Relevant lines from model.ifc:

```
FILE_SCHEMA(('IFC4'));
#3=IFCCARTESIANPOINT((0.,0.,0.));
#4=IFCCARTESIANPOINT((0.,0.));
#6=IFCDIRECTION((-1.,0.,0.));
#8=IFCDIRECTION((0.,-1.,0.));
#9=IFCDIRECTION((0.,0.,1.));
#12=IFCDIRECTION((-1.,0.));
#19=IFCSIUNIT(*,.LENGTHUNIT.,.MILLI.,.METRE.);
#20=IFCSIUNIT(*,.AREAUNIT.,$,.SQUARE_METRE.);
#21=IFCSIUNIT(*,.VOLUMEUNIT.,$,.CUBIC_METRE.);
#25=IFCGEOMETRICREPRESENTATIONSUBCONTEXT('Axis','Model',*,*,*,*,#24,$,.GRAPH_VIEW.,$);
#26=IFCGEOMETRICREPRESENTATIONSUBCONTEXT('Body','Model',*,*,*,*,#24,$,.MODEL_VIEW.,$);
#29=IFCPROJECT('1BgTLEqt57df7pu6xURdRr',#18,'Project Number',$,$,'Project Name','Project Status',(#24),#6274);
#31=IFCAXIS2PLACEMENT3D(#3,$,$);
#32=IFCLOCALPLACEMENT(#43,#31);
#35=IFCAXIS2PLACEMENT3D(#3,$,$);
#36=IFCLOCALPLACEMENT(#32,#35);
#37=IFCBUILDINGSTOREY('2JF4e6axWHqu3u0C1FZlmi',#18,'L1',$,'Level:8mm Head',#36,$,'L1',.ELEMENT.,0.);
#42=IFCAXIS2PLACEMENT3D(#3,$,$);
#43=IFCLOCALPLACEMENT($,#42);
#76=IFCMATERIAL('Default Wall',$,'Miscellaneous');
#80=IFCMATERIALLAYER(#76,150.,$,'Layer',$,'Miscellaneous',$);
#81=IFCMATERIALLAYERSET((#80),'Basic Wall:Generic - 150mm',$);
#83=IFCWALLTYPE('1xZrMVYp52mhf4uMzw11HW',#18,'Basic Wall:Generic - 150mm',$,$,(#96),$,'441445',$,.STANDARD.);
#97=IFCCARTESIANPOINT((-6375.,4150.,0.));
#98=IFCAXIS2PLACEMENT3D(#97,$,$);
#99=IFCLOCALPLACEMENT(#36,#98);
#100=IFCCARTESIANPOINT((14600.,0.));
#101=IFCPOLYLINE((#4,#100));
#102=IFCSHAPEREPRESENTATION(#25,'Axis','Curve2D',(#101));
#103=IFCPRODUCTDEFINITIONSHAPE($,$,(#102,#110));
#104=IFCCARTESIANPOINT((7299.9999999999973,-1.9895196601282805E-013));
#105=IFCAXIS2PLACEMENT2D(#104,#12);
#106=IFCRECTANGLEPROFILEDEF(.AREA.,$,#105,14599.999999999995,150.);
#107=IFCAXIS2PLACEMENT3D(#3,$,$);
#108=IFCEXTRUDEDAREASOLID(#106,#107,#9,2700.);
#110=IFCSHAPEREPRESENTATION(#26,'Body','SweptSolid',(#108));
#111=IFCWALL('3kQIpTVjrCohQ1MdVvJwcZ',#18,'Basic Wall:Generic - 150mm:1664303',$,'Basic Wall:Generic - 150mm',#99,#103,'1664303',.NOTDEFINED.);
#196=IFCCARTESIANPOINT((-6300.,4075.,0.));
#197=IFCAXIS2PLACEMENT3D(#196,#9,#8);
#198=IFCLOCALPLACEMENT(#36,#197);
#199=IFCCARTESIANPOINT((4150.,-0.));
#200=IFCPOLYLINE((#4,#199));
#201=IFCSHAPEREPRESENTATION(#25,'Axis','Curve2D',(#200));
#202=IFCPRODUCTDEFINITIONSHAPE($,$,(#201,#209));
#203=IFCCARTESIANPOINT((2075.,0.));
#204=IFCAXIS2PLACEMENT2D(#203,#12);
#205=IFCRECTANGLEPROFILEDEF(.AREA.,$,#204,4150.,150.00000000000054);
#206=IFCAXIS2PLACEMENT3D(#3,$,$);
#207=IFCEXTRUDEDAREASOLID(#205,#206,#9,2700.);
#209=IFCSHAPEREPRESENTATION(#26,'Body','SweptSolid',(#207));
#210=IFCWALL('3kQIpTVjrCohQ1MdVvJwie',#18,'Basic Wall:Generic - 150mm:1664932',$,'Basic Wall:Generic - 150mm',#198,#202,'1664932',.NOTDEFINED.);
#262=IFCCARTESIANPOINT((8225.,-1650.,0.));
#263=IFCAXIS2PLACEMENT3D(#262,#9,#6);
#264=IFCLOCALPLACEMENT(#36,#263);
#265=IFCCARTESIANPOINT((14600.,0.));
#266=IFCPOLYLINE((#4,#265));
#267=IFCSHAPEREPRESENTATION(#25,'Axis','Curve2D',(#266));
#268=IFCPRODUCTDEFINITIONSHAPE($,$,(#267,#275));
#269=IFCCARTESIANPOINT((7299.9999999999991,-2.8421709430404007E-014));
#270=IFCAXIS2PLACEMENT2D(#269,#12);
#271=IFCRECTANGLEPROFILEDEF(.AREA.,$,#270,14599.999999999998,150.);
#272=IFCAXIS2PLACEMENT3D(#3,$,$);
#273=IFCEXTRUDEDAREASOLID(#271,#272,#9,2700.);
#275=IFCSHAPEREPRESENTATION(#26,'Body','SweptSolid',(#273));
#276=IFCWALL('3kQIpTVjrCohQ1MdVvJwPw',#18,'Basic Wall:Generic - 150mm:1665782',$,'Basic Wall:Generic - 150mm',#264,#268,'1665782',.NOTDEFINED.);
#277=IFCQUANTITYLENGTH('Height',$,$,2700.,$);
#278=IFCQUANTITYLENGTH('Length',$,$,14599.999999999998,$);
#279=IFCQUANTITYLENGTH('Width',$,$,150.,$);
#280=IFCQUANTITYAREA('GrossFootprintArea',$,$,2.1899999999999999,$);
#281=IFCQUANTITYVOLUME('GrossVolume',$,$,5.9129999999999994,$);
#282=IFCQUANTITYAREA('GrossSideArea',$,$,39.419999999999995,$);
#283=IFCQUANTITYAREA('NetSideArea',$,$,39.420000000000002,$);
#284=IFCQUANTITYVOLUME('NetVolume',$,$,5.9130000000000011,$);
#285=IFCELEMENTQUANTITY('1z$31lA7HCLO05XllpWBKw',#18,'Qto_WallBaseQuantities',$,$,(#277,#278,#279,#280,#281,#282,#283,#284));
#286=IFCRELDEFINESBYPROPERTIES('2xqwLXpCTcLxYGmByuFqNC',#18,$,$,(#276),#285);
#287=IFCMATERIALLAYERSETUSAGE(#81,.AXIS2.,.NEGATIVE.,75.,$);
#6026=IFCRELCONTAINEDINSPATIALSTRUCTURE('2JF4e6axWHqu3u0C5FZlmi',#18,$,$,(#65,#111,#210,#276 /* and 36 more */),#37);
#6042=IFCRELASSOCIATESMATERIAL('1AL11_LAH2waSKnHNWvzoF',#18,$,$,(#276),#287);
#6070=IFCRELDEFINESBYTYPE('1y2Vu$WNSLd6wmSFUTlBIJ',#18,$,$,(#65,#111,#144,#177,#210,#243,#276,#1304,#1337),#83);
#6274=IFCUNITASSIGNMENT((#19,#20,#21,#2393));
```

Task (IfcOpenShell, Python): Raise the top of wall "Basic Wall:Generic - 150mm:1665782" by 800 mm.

```python
import ifcopenshell
import ifcopenshell.api.pset
import ifcopenshell.geom
import ifcopenshell.util.element
import ifcopenshell.util.representation
import ifcopenshell.util.shape
import ifcopenshell.util.unit

model = ifcopenshell.open("model.ifc")
unit_scale = ifcopenshell.util.unit.calculate_unit_scale(model)
area_scale = ifcopenshell.util.unit.calculate_unit_scale(model, "AREAUNIT")
volume_scale = ifcopenshell.util.unit.calculate_unit_scale(model, "VOLUMEUNIT")
settings = ifcopenshell.geom.settings()


def volume(element):
    """Net volume in cubic metres, openings subtracted."""
    shape = ifcopenshell.geom.create_shape(settings, element)
    return ifcopenshell.util.shape.get_volume(shape.geometry)


wall = model.by_id(276)
before = volume(wall)

body = ifcopenshell.util.representation.get_representation(wall, "Model", "Body")
solid = body.Items[0]
old_height = solid.Depth
solid.Depth += 800.0
after = volume(wall)
thickness = 0.15  # wall thickness in metres

# Update the stored height, areas and volumes.
qto = model.by_id(ifcopenshell.util.element.get_pset(wall, "Qto_WallBaseQuantities", should_inherit=False)["id"])
ifcopenshell.api.pset.edit_qto(model, qto=qto, properties={
    "Height": solid.Depth,
    "GrossVolume": ifcopenshell.util.element.get_pset(wall, "Qto_WallBaseQuantities", "GrossVolume") * solid.Depth / old_height,
    "GrossSideArea": ifcopenshell.util.element.get_pset(wall, "Qto_WallBaseQuantities", "GrossSideArea") * solid.Depth / old_height,
    "NetSideArea": after / thickness / area_scale,
    "NetVolume": after / volume_scale,
})

print(f"height {old_height:g} -> {solid.Depth:g}, volume {before:.3f} -> {after:.3f} m3")

model.write("model_edited.ifc")
```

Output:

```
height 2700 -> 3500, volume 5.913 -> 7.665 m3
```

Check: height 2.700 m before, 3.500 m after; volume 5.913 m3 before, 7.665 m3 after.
